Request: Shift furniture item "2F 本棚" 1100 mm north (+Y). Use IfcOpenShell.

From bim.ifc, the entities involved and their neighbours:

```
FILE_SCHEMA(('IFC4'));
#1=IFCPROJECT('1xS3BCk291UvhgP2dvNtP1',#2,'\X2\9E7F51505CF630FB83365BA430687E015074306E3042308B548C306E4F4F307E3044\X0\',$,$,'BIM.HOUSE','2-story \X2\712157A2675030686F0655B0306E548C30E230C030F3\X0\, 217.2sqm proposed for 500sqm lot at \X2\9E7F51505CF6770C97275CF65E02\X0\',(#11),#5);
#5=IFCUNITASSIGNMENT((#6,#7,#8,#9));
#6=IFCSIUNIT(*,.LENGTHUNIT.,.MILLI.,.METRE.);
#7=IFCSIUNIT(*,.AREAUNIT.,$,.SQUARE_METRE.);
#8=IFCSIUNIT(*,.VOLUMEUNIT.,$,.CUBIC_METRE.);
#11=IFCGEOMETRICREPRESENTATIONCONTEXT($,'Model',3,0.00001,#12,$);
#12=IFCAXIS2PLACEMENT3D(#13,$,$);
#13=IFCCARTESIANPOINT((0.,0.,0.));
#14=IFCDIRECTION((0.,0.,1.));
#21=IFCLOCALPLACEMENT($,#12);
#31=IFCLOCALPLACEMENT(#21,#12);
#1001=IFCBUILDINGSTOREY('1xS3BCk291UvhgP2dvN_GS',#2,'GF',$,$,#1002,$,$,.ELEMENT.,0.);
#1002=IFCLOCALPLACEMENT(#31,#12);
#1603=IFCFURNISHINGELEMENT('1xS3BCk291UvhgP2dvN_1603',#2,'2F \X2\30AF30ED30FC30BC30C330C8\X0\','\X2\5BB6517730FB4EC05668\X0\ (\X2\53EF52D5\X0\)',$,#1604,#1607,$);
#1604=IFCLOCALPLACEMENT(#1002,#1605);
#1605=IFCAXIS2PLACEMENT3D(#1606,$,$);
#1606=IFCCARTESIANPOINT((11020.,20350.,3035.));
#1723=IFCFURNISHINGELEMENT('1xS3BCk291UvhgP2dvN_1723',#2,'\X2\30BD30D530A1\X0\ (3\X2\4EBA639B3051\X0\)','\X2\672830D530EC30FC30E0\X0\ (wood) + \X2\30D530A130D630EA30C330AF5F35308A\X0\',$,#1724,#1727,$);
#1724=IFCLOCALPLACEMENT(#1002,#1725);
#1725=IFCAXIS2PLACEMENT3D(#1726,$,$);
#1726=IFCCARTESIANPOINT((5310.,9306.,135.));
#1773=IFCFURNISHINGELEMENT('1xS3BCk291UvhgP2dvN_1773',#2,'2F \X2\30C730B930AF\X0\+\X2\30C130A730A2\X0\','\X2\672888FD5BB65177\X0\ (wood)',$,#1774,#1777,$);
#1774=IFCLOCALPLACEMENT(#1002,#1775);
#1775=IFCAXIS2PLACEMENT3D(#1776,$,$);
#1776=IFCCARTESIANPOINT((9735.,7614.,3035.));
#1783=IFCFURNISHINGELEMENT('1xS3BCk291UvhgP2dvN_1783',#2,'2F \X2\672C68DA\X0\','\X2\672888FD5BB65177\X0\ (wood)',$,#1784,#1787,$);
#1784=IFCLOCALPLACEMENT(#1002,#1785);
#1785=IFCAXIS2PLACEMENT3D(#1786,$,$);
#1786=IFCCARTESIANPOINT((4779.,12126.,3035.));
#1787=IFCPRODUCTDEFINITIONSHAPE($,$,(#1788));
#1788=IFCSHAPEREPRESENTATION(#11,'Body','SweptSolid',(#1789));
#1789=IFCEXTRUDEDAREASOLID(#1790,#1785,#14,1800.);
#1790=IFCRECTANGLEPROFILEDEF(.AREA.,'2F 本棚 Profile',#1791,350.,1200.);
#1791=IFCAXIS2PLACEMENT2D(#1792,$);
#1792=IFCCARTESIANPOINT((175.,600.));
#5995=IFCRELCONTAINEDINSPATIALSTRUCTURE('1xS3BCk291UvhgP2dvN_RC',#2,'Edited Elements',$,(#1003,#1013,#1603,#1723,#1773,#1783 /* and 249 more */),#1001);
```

```python
import ifcopenshell
import ifcopenshell.api.geometry
import ifcopenshell.util.placement
import ifcopenshell.util.unit

model = ifcopenshell.open("bim.ifc")
unit_scale = ifcopenshell.util.unit.calculate_unit_scale(model)

item = model.by_guid("1xS3BCk291UvhgP2dvN_1783")
matrix = ifcopenshell.util.placement.get_local_placement(item.ObjectPlacement)
matrix[1, 3] += 1.1 / unit_scale
ifcopenshell.api.geometry.edit_object_placement(model, product=item, matrix=matrix, is_si=False)

print(ifcopenshell.util.placement.get_local_placement(item.ObjectPlacement).round(3) + 0.0)

model.write("bim_rev.ifc")
```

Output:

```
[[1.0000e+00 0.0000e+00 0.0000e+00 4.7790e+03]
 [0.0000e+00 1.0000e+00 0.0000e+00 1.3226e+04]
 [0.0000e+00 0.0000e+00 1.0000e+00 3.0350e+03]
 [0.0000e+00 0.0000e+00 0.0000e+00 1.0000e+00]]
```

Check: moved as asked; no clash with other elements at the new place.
